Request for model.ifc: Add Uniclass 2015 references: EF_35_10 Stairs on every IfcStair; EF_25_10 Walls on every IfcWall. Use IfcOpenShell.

First a look at what the model holds.

```python
import ifcopenshell

model = ifcopenshell.open("model.ifc")
print(model.schema)
print("classifications:", [c.Name for c in model.by_type("IfcClassification")])
for ifc_class in ("IfcDoor", "IfcRoof", "IfcStair", "IfcWall", "IfcWindow"):
    print(ifc_class, len(model.by_type(ifc_class)))
```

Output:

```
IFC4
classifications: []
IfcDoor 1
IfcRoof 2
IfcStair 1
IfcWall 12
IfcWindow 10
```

```python
import ifcopenshell
import ifcopenshell.api.classification

model = ifcopenshell.open("model.ifc")

system = ifcopenshell.api.classification.add_classification(model, classification="Uniclass 2015")

codes = {
    "IfcStair": ("EF_35_10", "Stairs"),
    "IfcWall": ("EF_25_10", "Walls"),
}
for ifc_class, (code, name) in codes.items():
    products = model.by_type(ifc_class)
    ifcopenshell.api.classification.add_reference(
        model, products=products, classification=system, identification=code, name=name
    )
    print(code, len(products))

model.write("model_edited.ifc")
```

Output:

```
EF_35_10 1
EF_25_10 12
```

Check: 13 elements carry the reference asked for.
